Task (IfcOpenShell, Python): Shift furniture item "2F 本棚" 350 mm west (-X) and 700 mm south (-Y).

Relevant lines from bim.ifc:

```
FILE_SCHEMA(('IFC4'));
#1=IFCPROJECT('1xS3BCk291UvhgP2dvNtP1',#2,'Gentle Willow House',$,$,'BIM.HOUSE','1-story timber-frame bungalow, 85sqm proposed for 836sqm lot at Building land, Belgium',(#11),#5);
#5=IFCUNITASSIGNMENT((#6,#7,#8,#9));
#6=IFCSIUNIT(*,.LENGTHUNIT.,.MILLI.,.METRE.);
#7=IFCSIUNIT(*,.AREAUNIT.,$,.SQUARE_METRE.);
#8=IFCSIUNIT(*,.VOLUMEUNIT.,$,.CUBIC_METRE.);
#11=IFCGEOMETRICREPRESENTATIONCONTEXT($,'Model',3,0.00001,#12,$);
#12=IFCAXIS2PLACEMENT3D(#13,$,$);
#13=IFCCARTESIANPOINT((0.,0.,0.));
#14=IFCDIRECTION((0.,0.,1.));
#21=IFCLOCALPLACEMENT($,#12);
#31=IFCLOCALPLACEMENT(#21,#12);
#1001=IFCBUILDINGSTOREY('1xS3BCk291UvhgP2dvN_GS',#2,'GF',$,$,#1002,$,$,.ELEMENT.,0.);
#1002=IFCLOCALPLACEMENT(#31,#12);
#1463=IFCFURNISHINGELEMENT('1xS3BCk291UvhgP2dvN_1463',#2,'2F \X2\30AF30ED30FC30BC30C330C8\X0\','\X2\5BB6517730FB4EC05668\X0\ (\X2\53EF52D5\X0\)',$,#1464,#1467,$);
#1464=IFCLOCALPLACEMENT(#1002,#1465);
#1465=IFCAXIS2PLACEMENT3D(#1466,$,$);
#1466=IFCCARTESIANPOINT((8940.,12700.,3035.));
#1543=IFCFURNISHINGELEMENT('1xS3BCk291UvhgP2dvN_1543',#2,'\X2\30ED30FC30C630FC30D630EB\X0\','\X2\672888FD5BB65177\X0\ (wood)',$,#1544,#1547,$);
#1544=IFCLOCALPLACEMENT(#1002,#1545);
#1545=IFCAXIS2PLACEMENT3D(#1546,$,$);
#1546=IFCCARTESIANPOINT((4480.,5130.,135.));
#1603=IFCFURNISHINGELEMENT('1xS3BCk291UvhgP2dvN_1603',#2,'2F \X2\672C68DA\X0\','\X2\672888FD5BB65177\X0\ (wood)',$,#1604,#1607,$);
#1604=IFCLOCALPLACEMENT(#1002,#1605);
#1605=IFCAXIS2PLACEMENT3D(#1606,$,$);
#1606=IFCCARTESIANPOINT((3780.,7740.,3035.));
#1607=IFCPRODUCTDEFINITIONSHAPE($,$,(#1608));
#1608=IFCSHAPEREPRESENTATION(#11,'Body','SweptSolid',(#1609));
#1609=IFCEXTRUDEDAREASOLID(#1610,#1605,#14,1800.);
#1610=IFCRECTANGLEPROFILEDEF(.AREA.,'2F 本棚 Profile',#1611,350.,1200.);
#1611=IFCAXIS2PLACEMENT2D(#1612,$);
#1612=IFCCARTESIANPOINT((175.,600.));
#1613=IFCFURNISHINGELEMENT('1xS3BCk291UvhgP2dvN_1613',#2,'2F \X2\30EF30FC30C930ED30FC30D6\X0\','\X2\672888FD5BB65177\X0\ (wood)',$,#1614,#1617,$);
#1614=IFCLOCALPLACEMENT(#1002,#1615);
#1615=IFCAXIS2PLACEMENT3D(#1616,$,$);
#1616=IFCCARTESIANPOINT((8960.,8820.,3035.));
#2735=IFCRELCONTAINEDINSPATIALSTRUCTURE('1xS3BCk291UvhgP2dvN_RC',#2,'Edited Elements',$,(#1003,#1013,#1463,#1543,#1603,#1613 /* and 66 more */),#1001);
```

```python
import ifcopenshell
import ifcopenshell.api.geometry
import ifcopenshell.util.placement
import ifcopenshell.util.unit

model = ifcopenshell.open("bim.ifc")
unit_scale = ifcopenshell.util.unit.calculate_unit_scale(model)

item = model.by_guid("1xS3BCk291UvhgP2dvN_1603")
matrix = ifcopenshell.util.placement.get_local_placement(item.ObjectPlacement)
matrix[0, 3] -= 0.35 / unit_scale
matrix[1, 3] -= 0.7 / unit_scale
ifcopenshell.api.geometry.edit_object_placement(model, product=item, matrix=matrix, is_si=False)

print(ifcopenshell.util.placement.get_local_placement(item.ObjectPlacement).round(3) + 0.0)

model.write("bim_v2.ifc")
```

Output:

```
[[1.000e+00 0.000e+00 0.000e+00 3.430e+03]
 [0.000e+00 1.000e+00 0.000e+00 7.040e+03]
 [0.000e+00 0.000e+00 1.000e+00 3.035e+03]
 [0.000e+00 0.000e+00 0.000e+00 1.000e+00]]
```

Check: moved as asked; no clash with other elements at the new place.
